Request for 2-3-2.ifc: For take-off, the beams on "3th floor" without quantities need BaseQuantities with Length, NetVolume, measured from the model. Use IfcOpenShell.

First a look at what the model holds.

```python
import ifcopenshell
import ifcopenshell.util.element
import ifcopenshell.util.unit

model = ifcopenshell.open("2-3-2.ifc")
print(model.schema)
for unit_type in ("LENGTHUNIT", "AREAUNIT", "VOLUMEUNIT"):
    print(unit_type, ifcopenshell.util.unit.calculate_unit_scale(model, unit_type))
storey = next(s for s in model.by_type("IfcBuildingStorey") if s.Name == "3th floor")
beams = [e for e in ifcopenshell.util.element.get_decomposition(storey) if e.is_a("IfcBeam")]
for e in sorted(beams, key=lambda e: e.id()):
    print(e.id(), e.is_a(), e.Name, list(ifcopenshell.util.element.get_psets(e, qtos_only=True)), sep=" | ")
```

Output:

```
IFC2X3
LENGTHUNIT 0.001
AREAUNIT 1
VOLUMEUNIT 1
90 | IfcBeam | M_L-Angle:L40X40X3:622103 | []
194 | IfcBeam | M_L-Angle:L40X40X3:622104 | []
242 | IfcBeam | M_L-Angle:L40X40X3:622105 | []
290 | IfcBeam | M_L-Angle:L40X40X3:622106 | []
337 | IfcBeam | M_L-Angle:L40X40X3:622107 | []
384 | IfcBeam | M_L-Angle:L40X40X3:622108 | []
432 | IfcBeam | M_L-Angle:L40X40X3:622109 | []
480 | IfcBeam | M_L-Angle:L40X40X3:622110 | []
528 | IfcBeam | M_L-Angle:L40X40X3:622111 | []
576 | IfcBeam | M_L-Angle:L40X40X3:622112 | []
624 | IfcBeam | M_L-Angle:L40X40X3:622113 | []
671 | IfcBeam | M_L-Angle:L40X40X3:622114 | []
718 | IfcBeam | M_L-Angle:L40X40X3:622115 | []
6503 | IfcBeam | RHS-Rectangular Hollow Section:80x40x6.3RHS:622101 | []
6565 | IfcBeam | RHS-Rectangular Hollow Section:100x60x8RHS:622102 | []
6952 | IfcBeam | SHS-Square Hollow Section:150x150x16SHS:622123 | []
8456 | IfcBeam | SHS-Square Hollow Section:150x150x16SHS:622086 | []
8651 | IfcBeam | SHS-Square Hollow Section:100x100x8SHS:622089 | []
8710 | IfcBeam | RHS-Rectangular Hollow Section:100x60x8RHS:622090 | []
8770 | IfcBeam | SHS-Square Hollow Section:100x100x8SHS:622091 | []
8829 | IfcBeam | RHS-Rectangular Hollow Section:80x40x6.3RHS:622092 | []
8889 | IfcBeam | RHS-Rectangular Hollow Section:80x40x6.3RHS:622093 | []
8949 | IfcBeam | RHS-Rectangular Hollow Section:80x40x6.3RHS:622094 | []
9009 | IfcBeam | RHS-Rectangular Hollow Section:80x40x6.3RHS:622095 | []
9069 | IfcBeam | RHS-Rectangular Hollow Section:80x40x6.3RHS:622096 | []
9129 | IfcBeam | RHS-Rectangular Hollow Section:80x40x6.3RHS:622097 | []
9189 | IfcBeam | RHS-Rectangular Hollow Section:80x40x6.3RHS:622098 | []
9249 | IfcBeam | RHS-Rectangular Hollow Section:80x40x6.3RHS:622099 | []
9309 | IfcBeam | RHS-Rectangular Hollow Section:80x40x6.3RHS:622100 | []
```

```python
import ifcopenshell
import ifcopenshell.api.pset
import ifcopenshell.geom
import ifcopenshell.util.element
import ifcopenshell.util.shape
import ifcopenshell.util.unit

model = ifcopenshell.open("2-3-2.ifc")
unit_scale = ifcopenshell.util.unit.calculate_unit_scale(model)
volume_scale = ifcopenshell.util.unit.calculate_unit_scale(model, "VOLUMEUNIT")
settings = ifcopenshell.geom.settings()

storey = next(s for s in model.by_type("IfcBuildingStorey") if s.Name == "3th floor")
beams = [e for e in ifcopenshell.util.element.get_decomposition(storey) if e.is_a("IfcBeam")]

for e in sorted(beams, key=lambda e: e.id()):
    if ifcopenshell.util.element.get_psets(e, qtos_only=True, should_inherit=False):
        continue
    # Geometry comes back in metres, in the element's own axes.
    shape = ifcopenshell.geom.create_shape(settings, e)
    values = {
        "Length": ifcopenshell.util.shape.get_max_xyz(shape.geometry) / unit_scale,
        "NetVolume": ifcopenshell.util.shape.get_volume(shape.geometry) / volume_scale,
    }
    qto = ifcopenshell.api.pset.add_qto(model, product=e, name="BaseQuantities")
    ifcopenshell.api.pset.edit_qto(model, qto=qto, properties=values)
    print(e.id(), {k: round(v, 3) for k, v in values.items()})

model.write("2-3-2_rev.ifc")
```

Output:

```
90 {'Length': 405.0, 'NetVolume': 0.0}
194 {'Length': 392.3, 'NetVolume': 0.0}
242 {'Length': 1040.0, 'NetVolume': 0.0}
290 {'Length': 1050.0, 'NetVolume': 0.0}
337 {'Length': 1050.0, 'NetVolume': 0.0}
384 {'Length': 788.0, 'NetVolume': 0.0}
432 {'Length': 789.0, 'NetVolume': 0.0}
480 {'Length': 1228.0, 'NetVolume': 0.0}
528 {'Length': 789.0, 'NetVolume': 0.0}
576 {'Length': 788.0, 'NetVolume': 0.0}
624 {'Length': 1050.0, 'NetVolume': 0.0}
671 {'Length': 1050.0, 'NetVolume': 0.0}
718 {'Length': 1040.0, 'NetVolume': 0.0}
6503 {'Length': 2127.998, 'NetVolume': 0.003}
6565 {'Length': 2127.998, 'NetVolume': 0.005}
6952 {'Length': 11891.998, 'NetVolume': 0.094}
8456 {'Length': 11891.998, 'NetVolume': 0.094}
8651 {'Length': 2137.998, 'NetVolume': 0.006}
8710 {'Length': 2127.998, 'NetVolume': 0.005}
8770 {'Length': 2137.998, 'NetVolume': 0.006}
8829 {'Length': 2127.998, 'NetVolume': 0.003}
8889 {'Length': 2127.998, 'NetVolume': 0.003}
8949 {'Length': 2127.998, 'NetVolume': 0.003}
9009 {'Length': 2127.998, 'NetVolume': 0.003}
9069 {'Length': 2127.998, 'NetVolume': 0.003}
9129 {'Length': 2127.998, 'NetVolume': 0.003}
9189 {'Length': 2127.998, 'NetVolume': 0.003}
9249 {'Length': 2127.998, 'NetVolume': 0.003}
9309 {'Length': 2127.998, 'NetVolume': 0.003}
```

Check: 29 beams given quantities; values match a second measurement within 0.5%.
